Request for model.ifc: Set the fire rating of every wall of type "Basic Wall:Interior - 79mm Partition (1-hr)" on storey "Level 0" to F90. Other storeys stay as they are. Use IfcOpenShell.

First a look at what the model holds.

```python
import ifcopenshell
import ifcopenshell.util.element

model = ifcopenshell.open("model.ifc")
print(model.schema)
storey = next(s for s in model.by_type("IfcBuildingStorey") if s.Name == "Level 0")
walls = [e for e in ifcopenshell.util.element.get_decomposition(storey) if e.is_a("IfcWall")]
seen = {}
for e in walls:
    element_type = ifcopenshell.util.element.get_type(e)
    key = (element_type.Name if element_type != e and element_type else None, ifcopenshell.util.element.get_pset(e, "Pset_WallCommon", "FireRating"))
    seen[key] = seen.get(key, 0) + 1
for (name, value), count in sorted(seen.items(), key=str):
    print(count, "x", name, "|", value)
```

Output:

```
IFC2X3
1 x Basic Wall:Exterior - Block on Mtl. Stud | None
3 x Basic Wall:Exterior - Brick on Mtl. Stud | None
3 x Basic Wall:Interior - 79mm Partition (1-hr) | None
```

```python
import ifcopenshell
import ifcopenshell.api.pset
import ifcopenshell.util.element

model = ifcopenshell.open("model.ifc")

storey = next(s for s in model.by_type("IfcBuildingStorey") if s.Name == "Level 0")
walls = [e for e in ifcopenshell.util.element.get_decomposition(storey) if e.is_a("IfcWall")]

count = 0
for e in walls:
    element_type = ifcopenshell.util.element.get_type(e)
    if element_type in (None, e) or element_type.Name != "Basic Wall:Interior - 79mm Partition (1-hr)":
        continue
    # add_pset returns the element's existing set when there is one.
    pset = ifcopenshell.api.pset.add_pset(model, product=e, name="Pset_WallCommon")
    ifcopenshell.api.pset.edit_pset(model, pset=pset, properties={"FireRating": "F90"})
    count += 1

print(count, "walls updated")

model.write("model_rev.ifc")
```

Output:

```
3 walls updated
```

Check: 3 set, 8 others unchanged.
